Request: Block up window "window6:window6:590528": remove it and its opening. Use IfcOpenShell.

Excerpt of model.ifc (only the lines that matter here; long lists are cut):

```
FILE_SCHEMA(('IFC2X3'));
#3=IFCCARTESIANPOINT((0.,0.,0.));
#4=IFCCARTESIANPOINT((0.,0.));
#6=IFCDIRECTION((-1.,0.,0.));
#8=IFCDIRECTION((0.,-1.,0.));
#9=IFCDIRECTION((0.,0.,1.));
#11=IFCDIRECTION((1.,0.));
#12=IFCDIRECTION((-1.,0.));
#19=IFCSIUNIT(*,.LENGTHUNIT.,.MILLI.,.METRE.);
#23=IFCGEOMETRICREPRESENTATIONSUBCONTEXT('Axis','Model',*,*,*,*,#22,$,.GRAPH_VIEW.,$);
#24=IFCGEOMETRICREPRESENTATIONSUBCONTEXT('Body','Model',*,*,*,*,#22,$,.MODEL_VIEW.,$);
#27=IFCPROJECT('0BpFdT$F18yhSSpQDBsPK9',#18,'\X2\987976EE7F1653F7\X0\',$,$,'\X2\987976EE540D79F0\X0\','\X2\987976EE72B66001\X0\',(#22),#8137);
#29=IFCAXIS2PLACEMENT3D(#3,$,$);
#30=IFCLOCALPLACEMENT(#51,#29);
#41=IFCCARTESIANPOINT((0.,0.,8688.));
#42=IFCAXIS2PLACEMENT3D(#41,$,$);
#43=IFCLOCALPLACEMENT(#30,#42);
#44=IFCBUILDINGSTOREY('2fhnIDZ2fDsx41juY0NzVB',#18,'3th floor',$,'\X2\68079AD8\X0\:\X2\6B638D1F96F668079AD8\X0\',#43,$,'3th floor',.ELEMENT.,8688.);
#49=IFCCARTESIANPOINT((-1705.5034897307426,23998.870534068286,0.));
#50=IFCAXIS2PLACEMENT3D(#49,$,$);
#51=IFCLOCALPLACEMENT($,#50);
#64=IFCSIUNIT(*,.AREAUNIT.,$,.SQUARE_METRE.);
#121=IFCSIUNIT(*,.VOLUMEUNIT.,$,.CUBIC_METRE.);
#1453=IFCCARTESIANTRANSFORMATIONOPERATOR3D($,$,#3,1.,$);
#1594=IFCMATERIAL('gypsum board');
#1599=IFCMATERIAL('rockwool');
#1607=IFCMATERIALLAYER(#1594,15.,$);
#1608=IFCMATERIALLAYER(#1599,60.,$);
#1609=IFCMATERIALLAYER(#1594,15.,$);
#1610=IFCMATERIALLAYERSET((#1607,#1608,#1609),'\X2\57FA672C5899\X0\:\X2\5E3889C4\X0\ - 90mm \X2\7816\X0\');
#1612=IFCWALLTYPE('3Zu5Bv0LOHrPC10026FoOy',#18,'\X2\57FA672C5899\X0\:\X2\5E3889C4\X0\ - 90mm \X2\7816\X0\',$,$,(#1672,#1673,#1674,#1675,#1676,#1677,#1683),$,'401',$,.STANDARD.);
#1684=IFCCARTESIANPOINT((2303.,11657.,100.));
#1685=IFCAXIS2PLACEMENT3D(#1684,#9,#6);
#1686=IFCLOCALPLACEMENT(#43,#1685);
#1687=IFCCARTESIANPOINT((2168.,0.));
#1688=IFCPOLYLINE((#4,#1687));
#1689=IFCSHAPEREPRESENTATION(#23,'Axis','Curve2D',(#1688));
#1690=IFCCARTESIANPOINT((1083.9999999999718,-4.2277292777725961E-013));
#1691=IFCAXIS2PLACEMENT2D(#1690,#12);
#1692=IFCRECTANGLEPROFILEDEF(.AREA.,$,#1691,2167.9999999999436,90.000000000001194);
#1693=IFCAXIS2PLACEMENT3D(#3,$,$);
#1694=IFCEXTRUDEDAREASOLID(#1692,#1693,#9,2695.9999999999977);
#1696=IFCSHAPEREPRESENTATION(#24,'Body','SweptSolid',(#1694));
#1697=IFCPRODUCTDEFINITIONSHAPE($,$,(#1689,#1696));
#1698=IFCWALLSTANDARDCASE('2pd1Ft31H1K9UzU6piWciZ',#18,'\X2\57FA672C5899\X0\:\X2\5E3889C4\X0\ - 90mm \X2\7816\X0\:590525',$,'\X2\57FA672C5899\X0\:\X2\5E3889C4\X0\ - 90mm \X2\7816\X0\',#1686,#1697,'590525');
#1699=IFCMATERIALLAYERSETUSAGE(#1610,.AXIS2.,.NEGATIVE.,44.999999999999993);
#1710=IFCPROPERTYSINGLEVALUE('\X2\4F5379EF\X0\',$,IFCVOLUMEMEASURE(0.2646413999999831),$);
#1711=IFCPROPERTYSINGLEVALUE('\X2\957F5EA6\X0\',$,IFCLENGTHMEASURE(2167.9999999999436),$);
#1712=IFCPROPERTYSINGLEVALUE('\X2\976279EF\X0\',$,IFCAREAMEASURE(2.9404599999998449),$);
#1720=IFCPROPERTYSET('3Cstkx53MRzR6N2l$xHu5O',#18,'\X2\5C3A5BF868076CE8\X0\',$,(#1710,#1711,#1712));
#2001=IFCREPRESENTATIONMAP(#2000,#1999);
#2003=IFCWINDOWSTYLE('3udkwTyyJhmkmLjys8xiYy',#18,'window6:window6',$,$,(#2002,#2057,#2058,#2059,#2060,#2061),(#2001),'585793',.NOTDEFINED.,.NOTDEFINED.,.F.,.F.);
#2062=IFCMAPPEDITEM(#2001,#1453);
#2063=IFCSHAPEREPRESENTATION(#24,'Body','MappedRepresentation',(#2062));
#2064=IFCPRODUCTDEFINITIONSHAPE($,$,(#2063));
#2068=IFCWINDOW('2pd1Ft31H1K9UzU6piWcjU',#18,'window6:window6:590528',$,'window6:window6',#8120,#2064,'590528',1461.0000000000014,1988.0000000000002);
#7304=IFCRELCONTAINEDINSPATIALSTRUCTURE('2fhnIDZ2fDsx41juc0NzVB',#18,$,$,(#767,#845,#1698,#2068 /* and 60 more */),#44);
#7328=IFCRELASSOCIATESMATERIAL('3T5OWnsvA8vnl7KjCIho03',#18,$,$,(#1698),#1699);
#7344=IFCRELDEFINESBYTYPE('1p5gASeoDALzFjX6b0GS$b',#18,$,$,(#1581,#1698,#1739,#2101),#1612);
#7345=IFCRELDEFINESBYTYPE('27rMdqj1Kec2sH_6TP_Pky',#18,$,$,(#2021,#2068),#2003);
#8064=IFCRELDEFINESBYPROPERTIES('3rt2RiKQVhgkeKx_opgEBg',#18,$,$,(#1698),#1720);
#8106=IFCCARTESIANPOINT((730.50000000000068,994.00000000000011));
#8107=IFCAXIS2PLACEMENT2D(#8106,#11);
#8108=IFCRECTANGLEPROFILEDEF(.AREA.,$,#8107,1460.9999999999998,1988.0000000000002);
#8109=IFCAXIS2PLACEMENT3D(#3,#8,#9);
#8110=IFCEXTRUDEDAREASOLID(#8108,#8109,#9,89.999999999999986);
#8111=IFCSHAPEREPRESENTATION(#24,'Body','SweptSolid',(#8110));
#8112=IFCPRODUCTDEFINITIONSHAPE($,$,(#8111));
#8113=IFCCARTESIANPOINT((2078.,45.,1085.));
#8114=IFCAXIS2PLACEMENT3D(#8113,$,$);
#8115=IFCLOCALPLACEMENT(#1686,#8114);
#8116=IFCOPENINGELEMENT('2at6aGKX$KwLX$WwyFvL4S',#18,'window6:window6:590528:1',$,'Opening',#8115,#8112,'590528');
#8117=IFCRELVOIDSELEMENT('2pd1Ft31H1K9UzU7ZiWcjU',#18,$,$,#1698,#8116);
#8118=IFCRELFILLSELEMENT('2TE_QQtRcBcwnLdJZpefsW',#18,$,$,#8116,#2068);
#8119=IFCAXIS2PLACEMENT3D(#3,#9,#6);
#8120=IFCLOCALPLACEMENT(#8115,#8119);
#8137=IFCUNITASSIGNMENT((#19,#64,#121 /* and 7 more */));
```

```python
import ifcopenshell
import ifcopenshell.api.feature
import ifcopenshell.api.pset
import ifcopenshell.api.root
import ifcopenshell.geom
import ifcopenshell.util.element
import ifcopenshell.util.shape
import ifcopenshell.util.unit

model = ifcopenshell.open("model.ifc")
area_scale = ifcopenshell.util.unit.calculate_unit_scale(model, "AREAUNIT")
volume_scale = ifcopenshell.util.unit.calculate_unit_scale(model, "VOLUMEUNIT")
settings = ifcopenshell.geom.settings()


def volume(element):
    """Net volume in cubic metres, openings subtracted."""
    shape = ifcopenshell.geom.create_shape(settings, element)
    return ifcopenshell.util.shape.get_volume(shape.geometry)


window = model.by_guid("2pd1Ft31H1K9UzU6piWcjU")
opening = window.FillsVoids[0].RelatingOpeningElement
wall = opening.VoidsElements[0].RelatingBuildingElement
before = volume(wall)

ifcopenshell.api.root.remove_product(model, product=window)
ifcopenshell.api.feature.remove_feature(model, feature=opening)

after = volume(wall)
thickness = 0.09  # wall thickness in metres

# Update the wall's stored quantities.
pset = model.by_id(ifcopenshell.util.element.get_pset(wall, "尺寸标注", should_inherit=False)["id"])
ifcopenshell.api.pset.edit_pset(model, pset=pset, properties={
    "体积": model.create_entity("IfcVolumeMeasure", after / volume_scale),
    "面积": model.create_entity("IfcAreaMeasure", after / thickness / area_scale),
})

print(f"wall volume {before:.3f} -> {after:.3f} m3")

model.write("model_edited.ifc")
```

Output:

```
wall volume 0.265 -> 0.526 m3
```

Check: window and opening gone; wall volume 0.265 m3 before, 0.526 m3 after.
